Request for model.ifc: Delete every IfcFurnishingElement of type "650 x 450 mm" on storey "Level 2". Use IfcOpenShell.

First a look at what the model holds.

```python
import ifcopenshell
import ifcopenshell.util.element

model = ifcopenshell.open("model.ifc")
print(model.schema)
storey = next(s for s in model.by_type("IfcBuildingStorey") if s.Name == "Level 2")
furniture = [e for e in ifcopenshell.util.element.get_decomposition(storey) if e.is_a("IfcFurnishingElement")]
seen = {}
for e in furniture:
    element_type = ifcopenshell.util.element.get_type(e)
    name = element_type.Name if element_type not in (None, e) else None
    seen[name] = seen.get(name, 0) + 1
for name, count in sorted(seen.items(), key=str):
    print(count, "x", name)
```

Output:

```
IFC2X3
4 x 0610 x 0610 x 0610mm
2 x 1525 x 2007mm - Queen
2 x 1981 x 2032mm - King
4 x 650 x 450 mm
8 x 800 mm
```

```python
import ifcopenshell
import ifcopenshell.api.root
import ifcopenshell.util.element

model = ifcopenshell.open("model.ifc")

storey = next(s for s in model.by_type("IfcBuildingStorey") if s.Name == "Level 2")
furniture = [e for e in ifcopenshell.util.element.get_decomposition(storey) if e.is_a("IfcFurnishingElement")]
targets = [e for e in furniture if (t := ifcopenshell.util.element.get_type(e)) not in (None, e) and t.Name == "650 x 450 mm"]

for e in targets:
    ifcopenshell.api.root.remove_product(model, product=e)
print(len(targets), "removed")

model.write("model_edited.ifc")
```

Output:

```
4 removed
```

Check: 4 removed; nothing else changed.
